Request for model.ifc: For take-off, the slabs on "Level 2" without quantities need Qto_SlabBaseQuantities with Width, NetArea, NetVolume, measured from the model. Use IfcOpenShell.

First a look at what the model holds.

```python
import ifcopenshell
import ifcopenshell.util.element
import ifcopenshell.util.unit

model = ifcopenshell.open("model.ifc")
print(model.schema)
for unit_type in ("LENGTHUNIT", "AREAUNIT", "VOLUMEUNIT"):
    print(unit_type, ifcopenshell.util.unit.calculate_unit_scale(model, unit_type))
storey = next(s for s in model.by_type("IfcBuildingStorey") if s.Name == "Level 2")
slabs = [e for e in ifcopenshell.util.element.get_decomposition(storey) if e.is_a("IfcSlab")]
for e in sorted(slabs, key=lambda e: e.id()):
    print(e.id(), e.is_a(), e.Name, list(ifcopenshell.util.element.get_psets(e, qtos_only=True)), sep=" | ")
```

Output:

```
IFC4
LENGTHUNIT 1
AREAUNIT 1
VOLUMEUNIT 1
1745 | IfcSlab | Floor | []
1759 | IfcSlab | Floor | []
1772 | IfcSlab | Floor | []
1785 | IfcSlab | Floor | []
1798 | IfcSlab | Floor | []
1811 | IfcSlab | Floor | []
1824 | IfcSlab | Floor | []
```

```python
import ifcopenshell
import ifcopenshell.api.pset
import ifcopenshell.geom
import ifcopenshell.util.element
import ifcopenshell.util.shape
import ifcopenshell.util.unit

model = ifcopenshell.open("model.ifc")
unit_scale = ifcopenshell.util.unit.calculate_unit_scale(model)
area_scale = ifcopenshell.util.unit.calculate_unit_scale(model, "AREAUNIT")
volume_scale = ifcopenshell.util.unit.calculate_unit_scale(model, "VOLUMEUNIT")
settings = ifcopenshell.geom.settings()

storey = next(s for s in model.by_type("IfcBuildingStorey") if s.Name == "Level 2")
slabs = [e for e in ifcopenshell.util.element.get_decomposition(storey) if e.is_a("IfcSlab")]

for e in sorted(slabs, key=lambda e: e.id()):
    if ifcopenshell.util.element.get_psets(e, qtos_only=True, should_inherit=False):
        continue
    # Geometry comes back in metres, in the element's own axes.
    shape = ifcopenshell.geom.create_shape(settings, e)
    values = {
        "Width": ifcopenshell.util.shape.get_z(shape.geometry) / unit_scale,
        "NetArea": ifcopenshell.util.shape.get_footprint_area(shape.geometry) / area_scale,
        "NetVolume": ifcopenshell.util.shape.get_volume(shape.geometry) / volume_scale,
    }
    qto = ifcopenshell.api.pset.add_qto(model, product=e, name="Qto_SlabBaseQuantities")
    ifcopenshell.api.pset.edit_qto(model, qto=qto, properties=values)
    print(e.id(), {k: round(v, 3) for k, v in values.items()})

model.write("model_rev.ifc")
```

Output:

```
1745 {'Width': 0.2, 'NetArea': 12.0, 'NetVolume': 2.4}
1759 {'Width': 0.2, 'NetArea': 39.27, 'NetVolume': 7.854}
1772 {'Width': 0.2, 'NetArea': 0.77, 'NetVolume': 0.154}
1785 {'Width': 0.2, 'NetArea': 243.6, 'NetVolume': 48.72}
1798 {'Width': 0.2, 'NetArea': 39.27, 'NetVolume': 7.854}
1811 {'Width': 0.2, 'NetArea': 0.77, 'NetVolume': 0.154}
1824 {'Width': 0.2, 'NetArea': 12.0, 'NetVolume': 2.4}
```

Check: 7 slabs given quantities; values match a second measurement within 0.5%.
